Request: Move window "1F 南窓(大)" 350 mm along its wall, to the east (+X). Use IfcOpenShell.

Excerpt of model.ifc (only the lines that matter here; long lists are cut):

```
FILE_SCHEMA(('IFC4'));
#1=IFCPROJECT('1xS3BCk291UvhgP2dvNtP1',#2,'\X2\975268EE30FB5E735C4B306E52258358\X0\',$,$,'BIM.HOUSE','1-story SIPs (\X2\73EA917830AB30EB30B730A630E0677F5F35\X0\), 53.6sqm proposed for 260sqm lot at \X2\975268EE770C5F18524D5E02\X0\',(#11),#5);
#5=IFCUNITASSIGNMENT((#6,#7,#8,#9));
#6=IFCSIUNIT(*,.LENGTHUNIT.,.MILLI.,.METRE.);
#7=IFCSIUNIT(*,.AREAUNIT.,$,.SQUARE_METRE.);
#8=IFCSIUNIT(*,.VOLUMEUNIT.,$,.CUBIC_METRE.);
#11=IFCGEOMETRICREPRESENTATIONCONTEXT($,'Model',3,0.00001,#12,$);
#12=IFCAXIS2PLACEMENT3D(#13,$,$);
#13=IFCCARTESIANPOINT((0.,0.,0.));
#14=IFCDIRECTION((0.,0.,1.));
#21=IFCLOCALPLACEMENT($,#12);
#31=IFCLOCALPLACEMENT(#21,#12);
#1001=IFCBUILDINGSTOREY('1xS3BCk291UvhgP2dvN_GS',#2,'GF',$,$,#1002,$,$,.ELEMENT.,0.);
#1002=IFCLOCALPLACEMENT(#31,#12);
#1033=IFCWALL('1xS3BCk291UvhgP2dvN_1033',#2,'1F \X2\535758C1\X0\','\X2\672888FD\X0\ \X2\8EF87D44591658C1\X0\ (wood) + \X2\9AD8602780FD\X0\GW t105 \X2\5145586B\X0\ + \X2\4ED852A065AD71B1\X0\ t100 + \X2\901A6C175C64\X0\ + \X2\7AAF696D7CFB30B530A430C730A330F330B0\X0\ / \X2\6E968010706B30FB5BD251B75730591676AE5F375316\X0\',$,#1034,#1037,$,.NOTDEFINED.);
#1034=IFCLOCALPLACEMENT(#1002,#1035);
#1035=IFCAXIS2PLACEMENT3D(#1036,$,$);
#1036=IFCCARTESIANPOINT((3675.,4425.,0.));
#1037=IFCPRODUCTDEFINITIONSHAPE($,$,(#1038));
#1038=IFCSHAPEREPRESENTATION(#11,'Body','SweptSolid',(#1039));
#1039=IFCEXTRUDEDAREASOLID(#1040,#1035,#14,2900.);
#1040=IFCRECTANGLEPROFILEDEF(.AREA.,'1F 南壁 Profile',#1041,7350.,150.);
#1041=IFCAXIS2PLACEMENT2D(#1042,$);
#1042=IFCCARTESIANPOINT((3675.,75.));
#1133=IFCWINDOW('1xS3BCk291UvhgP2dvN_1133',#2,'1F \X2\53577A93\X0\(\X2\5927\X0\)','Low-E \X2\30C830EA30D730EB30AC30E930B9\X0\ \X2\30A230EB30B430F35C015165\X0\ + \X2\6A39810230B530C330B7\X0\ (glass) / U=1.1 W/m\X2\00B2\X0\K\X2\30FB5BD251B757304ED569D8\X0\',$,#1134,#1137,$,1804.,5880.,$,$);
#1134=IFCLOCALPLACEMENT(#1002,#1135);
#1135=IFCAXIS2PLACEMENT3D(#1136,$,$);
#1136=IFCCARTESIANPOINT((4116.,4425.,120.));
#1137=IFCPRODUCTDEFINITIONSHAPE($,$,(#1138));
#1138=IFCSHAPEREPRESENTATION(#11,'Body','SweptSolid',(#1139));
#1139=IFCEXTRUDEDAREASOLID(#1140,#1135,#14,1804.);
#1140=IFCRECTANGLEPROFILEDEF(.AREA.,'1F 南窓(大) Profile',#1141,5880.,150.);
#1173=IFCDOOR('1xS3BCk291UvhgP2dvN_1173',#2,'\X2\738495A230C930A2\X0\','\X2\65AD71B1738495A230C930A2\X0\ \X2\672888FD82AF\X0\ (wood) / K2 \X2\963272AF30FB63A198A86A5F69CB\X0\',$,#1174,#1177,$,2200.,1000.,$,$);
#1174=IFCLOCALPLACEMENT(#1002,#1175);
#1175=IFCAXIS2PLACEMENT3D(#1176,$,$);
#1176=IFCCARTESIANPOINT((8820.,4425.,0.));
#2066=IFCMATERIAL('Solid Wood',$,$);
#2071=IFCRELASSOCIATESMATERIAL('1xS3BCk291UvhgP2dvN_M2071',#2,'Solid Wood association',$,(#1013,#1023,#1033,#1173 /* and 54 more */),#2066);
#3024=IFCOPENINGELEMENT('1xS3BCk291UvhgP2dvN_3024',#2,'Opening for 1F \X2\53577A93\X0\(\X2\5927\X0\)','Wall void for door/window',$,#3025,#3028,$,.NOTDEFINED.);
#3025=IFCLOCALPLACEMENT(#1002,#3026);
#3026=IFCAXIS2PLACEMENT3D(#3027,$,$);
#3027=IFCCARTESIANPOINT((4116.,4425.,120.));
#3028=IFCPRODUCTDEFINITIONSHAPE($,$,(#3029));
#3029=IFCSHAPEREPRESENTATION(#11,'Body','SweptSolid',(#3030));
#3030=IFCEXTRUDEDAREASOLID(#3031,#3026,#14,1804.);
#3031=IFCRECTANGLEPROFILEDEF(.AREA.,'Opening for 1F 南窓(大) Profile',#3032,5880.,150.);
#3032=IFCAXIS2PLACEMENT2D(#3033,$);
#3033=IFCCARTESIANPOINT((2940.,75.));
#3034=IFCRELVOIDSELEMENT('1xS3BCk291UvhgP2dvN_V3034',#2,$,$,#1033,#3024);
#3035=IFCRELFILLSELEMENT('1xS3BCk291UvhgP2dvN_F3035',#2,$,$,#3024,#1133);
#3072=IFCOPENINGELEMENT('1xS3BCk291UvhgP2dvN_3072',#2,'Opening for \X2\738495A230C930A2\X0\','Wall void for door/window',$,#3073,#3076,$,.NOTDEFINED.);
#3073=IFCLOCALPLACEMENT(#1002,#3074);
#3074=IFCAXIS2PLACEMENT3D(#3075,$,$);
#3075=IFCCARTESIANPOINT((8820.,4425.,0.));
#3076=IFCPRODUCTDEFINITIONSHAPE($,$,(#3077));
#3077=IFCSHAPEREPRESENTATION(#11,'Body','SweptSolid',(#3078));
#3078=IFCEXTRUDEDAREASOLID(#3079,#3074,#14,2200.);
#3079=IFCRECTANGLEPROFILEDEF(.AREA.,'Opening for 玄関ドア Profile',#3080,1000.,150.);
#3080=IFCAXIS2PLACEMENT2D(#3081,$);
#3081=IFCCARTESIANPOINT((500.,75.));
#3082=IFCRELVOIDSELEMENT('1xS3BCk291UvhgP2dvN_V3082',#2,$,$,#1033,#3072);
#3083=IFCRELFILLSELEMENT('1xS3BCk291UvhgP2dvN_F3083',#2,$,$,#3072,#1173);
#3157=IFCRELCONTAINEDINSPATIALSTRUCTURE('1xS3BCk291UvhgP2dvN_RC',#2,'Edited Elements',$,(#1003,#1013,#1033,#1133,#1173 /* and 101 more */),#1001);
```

```python
import ifcopenshell
import ifcopenshell.api.geometry
import ifcopenshell.util.placement
import ifcopenshell.util.unit

model = ifcopenshell.open("model.ifc")
unit_scale = ifcopenshell.util.unit.calculate_unit_scale(model)

window = model.by_id(1133)
opening = window.FillsVoids[0].RelatingOpeningElement
wall = opening.VoidsElements[0].RelatingBuildingElement

wall_matrix = ifcopenshell.util.placement.get_local_placement(wall.ObjectPlacement)
shift = wall_matrix[:3, 0] * 0.35 / unit_scale
before = ifcopenshell.util.placement.get_local_placement(window.ObjectPlacement)[:3, 3].copy()

# The window is not placed relative to its opening, so move both.
for product in (opening, window):
    matrix = ifcopenshell.util.placement.get_local_placement(product.ObjectPlacement)
    matrix[:3, 3] += shift
    ifcopenshell.api.geometry.edit_object_placement(model, product=product, matrix=matrix, is_si=False)

after = ifcopenshell.util.placement.get_local_placement(window.ObjectPlacement)[:3, 3]
print("window moved by", (after - before).round(3) + 0.0)

model.write("model-out.ifc")
```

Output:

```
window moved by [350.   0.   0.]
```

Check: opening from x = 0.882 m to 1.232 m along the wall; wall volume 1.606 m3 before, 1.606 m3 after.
